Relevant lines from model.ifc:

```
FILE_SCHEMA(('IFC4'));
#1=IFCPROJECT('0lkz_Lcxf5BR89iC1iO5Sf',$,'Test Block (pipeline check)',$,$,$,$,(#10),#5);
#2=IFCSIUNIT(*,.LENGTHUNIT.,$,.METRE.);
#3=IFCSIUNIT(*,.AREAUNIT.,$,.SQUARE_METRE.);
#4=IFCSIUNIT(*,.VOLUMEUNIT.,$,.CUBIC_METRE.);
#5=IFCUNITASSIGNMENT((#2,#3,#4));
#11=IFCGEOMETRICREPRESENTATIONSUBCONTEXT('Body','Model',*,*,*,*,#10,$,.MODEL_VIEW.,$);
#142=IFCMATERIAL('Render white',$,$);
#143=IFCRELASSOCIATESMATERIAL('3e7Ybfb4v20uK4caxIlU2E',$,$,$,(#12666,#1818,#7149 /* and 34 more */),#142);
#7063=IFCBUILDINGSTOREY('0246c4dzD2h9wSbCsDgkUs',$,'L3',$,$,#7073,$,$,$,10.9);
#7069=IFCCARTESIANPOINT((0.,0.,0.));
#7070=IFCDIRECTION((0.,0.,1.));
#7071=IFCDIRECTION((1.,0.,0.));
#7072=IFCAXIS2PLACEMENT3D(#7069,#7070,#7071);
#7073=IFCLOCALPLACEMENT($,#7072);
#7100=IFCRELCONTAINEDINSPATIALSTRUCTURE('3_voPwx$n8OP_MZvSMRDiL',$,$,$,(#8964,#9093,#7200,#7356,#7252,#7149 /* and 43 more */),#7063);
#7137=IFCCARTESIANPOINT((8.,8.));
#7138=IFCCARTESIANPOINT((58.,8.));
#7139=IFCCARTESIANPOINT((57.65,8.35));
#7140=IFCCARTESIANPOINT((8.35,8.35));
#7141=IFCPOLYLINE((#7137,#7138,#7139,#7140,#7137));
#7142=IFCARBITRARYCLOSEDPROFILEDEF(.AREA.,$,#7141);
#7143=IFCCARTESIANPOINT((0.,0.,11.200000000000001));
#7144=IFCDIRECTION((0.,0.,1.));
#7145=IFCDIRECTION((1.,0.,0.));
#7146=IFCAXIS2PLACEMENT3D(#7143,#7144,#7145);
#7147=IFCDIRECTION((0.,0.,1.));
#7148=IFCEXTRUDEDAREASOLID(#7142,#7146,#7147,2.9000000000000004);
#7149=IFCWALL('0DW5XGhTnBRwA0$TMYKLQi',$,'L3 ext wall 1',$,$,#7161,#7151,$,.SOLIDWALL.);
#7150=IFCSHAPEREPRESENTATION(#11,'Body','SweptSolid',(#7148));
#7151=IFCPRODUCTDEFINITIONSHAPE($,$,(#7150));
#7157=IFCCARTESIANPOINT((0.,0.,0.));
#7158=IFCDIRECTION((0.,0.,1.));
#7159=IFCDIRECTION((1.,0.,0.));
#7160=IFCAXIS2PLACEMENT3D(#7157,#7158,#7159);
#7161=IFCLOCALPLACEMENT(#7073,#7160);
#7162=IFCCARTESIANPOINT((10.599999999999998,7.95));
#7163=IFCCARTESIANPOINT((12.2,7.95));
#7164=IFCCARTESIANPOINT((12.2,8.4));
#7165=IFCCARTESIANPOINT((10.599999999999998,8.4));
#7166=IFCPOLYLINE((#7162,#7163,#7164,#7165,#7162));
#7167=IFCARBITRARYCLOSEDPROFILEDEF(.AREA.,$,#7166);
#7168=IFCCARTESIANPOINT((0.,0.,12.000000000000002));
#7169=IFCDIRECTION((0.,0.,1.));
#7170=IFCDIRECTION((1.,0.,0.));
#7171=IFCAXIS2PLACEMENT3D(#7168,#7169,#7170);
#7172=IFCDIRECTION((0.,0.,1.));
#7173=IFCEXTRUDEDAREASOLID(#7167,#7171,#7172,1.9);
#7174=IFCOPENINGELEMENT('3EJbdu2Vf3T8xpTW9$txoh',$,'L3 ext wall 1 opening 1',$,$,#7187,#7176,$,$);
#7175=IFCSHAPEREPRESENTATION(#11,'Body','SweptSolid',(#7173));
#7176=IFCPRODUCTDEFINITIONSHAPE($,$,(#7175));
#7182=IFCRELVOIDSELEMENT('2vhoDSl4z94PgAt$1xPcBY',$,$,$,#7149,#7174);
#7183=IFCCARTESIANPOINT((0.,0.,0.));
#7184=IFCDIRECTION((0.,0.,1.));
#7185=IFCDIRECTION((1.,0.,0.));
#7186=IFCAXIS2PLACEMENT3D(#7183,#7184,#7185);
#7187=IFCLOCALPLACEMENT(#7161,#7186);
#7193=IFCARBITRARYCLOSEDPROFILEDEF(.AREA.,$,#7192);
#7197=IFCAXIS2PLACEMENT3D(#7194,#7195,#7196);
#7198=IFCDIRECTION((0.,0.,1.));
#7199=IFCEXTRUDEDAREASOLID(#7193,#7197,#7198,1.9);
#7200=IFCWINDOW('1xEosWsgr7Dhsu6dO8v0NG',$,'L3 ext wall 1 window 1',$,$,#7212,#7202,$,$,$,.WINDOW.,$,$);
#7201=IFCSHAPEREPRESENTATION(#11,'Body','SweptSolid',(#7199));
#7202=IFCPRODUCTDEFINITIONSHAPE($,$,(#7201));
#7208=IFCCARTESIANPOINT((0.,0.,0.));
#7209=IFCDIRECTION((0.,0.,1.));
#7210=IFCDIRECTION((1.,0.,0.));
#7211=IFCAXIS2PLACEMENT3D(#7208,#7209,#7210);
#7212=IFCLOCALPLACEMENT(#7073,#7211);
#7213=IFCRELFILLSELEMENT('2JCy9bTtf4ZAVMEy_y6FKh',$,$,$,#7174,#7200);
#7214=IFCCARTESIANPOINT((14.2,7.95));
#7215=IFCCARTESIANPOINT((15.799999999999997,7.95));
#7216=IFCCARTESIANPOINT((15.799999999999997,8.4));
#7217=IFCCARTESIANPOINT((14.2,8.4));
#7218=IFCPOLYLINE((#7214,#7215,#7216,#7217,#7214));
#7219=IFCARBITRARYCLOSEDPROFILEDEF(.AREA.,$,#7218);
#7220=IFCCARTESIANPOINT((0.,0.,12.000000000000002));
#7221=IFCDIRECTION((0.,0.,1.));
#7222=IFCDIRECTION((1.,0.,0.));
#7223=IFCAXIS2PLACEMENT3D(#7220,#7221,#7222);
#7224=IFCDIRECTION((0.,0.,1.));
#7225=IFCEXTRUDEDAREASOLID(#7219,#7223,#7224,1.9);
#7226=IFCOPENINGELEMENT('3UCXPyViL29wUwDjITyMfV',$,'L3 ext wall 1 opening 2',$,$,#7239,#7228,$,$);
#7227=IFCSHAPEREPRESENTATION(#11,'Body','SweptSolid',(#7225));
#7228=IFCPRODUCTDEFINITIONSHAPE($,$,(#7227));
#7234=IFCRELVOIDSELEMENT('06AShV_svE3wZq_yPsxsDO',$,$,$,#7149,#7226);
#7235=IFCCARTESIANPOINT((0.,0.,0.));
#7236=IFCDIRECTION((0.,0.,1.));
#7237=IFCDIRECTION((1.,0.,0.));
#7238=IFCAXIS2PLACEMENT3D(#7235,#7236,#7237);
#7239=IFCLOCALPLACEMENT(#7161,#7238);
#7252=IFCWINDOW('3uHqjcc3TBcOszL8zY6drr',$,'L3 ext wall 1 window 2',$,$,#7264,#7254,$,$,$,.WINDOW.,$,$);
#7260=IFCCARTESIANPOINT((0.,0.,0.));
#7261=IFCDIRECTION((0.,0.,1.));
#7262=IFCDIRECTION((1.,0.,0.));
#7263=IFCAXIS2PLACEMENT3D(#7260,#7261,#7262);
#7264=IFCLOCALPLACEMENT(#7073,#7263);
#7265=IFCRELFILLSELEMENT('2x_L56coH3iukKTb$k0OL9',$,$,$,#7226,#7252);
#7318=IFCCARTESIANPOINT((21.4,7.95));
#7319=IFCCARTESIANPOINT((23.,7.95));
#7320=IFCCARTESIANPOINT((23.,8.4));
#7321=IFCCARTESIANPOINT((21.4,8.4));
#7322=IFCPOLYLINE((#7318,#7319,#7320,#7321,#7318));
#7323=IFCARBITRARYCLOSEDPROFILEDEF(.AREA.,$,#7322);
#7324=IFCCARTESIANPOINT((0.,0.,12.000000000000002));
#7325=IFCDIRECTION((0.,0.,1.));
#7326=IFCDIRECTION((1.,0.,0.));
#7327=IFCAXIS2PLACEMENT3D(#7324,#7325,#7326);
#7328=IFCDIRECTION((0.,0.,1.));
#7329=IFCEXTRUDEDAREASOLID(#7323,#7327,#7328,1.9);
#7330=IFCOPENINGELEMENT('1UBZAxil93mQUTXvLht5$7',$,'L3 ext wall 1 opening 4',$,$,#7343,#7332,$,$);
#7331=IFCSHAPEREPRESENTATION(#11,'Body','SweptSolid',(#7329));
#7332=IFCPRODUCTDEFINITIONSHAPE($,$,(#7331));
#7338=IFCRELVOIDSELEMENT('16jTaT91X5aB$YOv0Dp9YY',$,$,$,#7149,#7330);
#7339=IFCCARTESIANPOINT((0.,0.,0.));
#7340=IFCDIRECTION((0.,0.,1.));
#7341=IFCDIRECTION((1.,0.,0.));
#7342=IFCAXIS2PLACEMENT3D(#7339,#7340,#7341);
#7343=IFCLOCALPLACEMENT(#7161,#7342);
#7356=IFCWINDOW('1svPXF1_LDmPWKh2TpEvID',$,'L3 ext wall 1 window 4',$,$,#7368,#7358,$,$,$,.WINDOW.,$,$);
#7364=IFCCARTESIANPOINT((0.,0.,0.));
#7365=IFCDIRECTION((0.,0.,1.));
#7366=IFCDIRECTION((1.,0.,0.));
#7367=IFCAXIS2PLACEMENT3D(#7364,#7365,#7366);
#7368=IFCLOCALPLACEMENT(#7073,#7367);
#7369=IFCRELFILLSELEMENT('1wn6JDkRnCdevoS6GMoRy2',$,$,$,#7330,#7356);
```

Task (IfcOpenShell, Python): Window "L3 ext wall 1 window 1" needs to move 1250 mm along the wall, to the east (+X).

```python
import ifcopenshell
import ifcopenshell.api.geometry
import ifcopenshell.util.placement
import ifcopenshell.util.unit

model = ifcopenshell.open("model.ifc")
unit_scale = ifcopenshell.util.unit.calculate_unit_scale(model)

window = model.by_id(7200)
opening = window.FillsVoids[0].RelatingOpeningElement
wall = opening.VoidsElements[0].RelatingBuildingElement

wall_matrix = ifcopenshell.util.placement.get_local_placement(wall.ObjectPlacement)
shift = wall_matrix[:3, 0] * 1.25 / unit_scale
before = ifcopenshell.util.placement.get_local_placement(window.ObjectPlacement)[:3, 3].copy()

# The window is not placed relative to its opening, so move both.
for product in (opening, window):
    matrix = ifcopenshell.util.placement.get_local_placement(product.ObjectPlacement)
    matrix[:3, 3] += shift
    ifcopenshell.api.geometry.edit_object_placement(model, product=product, matrix=matrix, is_si=False)

after = ifcopenshell.util.placement.get_local_placement(window.ObjectPlacement)[:3, 3]
print("window moved by", (after - before).round(3) + 0.0)

model.write("model-out.ifc")
```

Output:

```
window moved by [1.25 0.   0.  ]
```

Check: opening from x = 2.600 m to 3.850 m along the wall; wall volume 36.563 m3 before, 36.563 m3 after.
